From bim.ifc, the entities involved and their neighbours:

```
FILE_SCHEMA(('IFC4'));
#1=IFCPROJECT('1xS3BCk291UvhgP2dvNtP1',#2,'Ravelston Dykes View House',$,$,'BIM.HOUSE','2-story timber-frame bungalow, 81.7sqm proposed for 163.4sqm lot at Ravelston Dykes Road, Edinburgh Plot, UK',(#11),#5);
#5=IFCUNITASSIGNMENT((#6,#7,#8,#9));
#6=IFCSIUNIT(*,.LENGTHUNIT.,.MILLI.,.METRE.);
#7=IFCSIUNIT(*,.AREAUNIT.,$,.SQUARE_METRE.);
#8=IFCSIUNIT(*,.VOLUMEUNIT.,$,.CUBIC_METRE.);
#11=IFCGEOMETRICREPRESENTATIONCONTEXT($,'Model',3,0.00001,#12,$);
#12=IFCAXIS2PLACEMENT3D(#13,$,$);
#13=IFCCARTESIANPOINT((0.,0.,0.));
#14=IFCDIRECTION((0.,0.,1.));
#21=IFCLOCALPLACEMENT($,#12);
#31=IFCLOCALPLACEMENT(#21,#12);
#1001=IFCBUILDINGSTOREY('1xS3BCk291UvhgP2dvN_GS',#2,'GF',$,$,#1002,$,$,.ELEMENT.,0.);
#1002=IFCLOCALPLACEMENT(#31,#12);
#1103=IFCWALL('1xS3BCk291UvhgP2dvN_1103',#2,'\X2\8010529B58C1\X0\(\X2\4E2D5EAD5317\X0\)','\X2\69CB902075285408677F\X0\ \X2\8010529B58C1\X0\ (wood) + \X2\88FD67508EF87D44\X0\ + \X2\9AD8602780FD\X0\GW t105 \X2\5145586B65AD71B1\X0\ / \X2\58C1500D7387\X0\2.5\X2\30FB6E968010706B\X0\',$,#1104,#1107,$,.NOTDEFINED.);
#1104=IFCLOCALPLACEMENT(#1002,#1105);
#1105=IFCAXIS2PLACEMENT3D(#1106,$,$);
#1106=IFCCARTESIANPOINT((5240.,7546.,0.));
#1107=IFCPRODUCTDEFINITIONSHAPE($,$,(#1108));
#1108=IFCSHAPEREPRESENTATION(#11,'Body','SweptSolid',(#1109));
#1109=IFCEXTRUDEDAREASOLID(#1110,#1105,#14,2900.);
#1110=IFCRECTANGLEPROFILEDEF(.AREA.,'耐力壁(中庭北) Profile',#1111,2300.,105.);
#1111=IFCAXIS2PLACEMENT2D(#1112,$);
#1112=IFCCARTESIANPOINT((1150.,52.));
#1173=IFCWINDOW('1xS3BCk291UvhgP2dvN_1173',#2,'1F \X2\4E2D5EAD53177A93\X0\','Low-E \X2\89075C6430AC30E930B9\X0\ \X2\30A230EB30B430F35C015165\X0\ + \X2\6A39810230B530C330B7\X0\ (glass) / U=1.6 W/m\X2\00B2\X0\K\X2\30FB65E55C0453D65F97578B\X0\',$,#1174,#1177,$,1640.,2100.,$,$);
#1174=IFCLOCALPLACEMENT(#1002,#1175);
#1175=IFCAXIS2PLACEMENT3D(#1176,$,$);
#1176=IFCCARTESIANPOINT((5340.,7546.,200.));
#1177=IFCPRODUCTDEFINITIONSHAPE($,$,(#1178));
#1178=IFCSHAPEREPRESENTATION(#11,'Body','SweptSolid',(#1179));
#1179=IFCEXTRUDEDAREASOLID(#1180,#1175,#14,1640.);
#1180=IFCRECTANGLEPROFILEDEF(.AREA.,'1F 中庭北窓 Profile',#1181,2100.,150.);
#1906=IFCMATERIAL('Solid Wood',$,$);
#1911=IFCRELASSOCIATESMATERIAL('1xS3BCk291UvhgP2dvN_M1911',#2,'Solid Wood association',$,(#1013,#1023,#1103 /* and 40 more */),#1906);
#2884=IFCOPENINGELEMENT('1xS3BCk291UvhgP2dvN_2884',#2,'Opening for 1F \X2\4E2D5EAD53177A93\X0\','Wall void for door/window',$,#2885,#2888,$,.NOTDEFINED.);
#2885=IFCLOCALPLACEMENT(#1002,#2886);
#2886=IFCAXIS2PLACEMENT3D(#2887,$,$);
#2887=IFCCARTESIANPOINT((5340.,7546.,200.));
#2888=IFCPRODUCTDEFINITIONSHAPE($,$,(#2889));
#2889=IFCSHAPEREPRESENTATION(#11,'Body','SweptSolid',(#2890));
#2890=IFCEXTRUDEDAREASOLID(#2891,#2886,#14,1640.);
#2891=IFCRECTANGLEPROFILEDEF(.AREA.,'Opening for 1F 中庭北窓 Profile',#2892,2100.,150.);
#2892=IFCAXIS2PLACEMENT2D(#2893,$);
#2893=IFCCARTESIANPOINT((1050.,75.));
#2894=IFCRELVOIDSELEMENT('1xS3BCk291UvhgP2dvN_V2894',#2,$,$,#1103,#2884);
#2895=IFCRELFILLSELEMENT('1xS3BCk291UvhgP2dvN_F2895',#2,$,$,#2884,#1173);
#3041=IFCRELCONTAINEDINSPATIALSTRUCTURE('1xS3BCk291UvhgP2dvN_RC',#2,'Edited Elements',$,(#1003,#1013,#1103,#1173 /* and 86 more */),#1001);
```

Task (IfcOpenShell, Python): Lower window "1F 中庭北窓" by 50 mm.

```python
import numpy as np
import ifcopenshell
import ifcopenshell.api.geometry
import ifcopenshell.util.placement
import ifcopenshell.util.unit

model = ifcopenshell.open("bim.ifc")
unit_scale = ifcopenshell.util.unit.calculate_unit_scale(model)

window = model.by_id(1173)
opening = window.FillsVoids[0].RelatingOpeningElement
dz = -50.0

shift = np.array([0.0, 0.0, dz])
# The window is not placed relative to its opening, so move both.
for product in (opening, window):
    matrix = ifcopenshell.util.placement.get_local_placement(product.ObjectPlacement)
    matrix[:3, 3] += shift
    ifcopenshell.api.geometry.edit_object_placement(model, product=product, matrix=matrix, is_si=False)

print(f"moved by {dz * unit_scale:+.3f} m")

model.write("bim-out.ifc")
```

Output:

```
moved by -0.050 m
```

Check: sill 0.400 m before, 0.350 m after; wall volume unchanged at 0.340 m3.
